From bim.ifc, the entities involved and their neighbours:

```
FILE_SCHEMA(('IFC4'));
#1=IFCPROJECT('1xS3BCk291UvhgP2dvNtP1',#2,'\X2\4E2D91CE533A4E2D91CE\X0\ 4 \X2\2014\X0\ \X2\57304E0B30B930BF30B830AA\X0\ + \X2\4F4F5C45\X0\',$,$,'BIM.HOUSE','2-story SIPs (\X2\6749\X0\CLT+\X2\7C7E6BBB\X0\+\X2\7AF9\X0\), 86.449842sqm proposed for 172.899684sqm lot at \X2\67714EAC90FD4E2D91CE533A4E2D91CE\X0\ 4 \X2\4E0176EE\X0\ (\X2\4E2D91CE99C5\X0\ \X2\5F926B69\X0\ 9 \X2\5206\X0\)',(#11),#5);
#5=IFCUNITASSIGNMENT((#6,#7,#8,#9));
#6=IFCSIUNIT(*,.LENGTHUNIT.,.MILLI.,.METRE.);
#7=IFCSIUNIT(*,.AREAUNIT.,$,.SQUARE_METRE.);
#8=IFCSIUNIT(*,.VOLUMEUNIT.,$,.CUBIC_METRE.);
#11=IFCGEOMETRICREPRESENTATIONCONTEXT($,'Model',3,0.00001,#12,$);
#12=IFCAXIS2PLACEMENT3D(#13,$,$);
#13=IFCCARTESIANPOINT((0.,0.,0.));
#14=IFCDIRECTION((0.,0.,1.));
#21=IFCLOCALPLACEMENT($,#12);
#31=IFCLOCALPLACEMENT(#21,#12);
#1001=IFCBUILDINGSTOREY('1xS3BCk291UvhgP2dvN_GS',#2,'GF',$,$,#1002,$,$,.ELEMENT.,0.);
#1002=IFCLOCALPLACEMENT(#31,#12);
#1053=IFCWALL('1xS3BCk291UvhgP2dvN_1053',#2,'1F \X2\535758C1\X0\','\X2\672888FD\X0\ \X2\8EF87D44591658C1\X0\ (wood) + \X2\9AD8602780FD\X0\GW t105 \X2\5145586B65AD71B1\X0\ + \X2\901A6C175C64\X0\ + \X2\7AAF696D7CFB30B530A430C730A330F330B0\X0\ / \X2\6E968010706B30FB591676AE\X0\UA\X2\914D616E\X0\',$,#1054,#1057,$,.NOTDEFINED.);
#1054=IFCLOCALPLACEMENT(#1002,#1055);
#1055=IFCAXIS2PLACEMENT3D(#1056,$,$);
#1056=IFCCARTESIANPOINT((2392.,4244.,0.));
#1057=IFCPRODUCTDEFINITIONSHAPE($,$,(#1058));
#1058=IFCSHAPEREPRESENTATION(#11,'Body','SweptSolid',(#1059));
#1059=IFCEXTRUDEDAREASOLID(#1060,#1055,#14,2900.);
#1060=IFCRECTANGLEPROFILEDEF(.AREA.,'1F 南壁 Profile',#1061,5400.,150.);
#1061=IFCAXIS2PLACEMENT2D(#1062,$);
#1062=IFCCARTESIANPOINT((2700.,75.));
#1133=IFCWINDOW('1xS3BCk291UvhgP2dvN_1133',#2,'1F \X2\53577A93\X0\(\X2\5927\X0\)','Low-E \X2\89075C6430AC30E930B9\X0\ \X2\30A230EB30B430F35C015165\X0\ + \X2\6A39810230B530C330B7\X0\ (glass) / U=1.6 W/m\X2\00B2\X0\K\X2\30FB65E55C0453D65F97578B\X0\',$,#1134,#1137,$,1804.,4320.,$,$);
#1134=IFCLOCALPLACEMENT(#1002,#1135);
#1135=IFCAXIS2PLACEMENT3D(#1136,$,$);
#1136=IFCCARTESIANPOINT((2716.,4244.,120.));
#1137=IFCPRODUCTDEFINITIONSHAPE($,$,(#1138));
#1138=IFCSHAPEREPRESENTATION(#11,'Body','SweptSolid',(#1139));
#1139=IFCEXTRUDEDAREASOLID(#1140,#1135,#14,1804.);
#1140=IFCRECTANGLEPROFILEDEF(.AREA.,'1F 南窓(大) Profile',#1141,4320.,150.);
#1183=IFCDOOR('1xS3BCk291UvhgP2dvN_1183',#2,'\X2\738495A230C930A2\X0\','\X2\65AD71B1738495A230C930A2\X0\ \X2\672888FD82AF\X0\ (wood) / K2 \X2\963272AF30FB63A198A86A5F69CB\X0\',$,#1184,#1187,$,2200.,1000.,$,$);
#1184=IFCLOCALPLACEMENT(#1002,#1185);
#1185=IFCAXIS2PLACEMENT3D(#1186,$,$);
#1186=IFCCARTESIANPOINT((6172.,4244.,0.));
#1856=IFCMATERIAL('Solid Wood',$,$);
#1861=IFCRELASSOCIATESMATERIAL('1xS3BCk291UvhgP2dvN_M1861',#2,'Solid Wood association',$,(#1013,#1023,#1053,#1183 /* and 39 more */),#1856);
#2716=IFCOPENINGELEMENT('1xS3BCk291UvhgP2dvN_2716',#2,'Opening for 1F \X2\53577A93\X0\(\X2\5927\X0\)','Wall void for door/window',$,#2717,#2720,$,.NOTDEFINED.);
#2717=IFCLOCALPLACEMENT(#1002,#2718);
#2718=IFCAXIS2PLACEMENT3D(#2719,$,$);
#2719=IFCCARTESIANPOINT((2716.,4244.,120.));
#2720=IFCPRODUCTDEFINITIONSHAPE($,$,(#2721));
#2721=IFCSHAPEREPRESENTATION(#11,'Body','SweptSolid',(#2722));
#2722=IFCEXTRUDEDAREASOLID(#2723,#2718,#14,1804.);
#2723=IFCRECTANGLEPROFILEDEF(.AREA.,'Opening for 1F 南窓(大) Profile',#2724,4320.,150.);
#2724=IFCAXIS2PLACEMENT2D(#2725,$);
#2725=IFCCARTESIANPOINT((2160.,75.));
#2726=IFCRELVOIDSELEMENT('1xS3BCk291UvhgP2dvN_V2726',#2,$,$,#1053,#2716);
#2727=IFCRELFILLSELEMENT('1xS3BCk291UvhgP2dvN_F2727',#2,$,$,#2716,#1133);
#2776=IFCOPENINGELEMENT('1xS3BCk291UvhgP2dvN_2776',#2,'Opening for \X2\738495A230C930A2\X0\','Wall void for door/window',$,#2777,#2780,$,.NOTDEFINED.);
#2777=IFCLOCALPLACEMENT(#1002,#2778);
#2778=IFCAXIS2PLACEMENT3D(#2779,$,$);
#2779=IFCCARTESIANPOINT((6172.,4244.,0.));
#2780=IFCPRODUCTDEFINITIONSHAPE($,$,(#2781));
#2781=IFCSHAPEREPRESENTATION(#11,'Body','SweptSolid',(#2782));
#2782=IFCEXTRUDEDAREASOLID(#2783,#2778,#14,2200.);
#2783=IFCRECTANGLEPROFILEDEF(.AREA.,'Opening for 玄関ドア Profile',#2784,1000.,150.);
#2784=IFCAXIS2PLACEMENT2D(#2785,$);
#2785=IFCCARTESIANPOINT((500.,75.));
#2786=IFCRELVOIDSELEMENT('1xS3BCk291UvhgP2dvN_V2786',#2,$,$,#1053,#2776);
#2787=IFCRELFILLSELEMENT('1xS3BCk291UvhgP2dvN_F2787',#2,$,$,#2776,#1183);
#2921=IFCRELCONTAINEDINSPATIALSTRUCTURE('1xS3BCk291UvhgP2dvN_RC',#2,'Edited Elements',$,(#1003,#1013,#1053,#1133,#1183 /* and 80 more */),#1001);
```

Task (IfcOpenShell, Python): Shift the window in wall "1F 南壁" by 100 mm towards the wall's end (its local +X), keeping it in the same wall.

```python
import ifcopenshell
import ifcopenshell.api.geometry
import ifcopenshell.util.placement
import ifcopenshell.util.unit

model = ifcopenshell.open("bim.ifc")
unit_scale = ifcopenshell.util.unit.calculate_unit_scale(model)

window = model.by_guid("1xS3BCk291UvhgP2dvN_1133")
opening = window.FillsVoids[0].RelatingOpeningElement
wall = opening.VoidsElements[0].RelatingBuildingElement

wall_matrix = ifcopenshell.util.placement.get_local_placement(wall.ObjectPlacement)
shift = wall_matrix[:3, 0] * 0.1 / unit_scale
before = ifcopenshell.util.placement.get_local_placement(window.ObjectPlacement)[:3, 3].copy()

# The window is not placed relative to its opening, so move both.
for product in (opening, window):
    matrix = ifcopenshell.util.placement.get_local_placement(product.ObjectPlacement)
    matrix[:3, 3] += shift
    ifcopenshell.api.geometry.edit_object_placement(model, product=product, matrix=matrix, is_si=False)

after = ifcopenshell.util.placement.get_local_placement(window.ObjectPlacement)[:3, 3]
print("window moved by", (after - before).round(3) + 0.0)

model.write("bim_rev.ifc")
```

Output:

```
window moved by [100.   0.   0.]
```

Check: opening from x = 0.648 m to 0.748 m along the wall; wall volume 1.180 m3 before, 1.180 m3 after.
